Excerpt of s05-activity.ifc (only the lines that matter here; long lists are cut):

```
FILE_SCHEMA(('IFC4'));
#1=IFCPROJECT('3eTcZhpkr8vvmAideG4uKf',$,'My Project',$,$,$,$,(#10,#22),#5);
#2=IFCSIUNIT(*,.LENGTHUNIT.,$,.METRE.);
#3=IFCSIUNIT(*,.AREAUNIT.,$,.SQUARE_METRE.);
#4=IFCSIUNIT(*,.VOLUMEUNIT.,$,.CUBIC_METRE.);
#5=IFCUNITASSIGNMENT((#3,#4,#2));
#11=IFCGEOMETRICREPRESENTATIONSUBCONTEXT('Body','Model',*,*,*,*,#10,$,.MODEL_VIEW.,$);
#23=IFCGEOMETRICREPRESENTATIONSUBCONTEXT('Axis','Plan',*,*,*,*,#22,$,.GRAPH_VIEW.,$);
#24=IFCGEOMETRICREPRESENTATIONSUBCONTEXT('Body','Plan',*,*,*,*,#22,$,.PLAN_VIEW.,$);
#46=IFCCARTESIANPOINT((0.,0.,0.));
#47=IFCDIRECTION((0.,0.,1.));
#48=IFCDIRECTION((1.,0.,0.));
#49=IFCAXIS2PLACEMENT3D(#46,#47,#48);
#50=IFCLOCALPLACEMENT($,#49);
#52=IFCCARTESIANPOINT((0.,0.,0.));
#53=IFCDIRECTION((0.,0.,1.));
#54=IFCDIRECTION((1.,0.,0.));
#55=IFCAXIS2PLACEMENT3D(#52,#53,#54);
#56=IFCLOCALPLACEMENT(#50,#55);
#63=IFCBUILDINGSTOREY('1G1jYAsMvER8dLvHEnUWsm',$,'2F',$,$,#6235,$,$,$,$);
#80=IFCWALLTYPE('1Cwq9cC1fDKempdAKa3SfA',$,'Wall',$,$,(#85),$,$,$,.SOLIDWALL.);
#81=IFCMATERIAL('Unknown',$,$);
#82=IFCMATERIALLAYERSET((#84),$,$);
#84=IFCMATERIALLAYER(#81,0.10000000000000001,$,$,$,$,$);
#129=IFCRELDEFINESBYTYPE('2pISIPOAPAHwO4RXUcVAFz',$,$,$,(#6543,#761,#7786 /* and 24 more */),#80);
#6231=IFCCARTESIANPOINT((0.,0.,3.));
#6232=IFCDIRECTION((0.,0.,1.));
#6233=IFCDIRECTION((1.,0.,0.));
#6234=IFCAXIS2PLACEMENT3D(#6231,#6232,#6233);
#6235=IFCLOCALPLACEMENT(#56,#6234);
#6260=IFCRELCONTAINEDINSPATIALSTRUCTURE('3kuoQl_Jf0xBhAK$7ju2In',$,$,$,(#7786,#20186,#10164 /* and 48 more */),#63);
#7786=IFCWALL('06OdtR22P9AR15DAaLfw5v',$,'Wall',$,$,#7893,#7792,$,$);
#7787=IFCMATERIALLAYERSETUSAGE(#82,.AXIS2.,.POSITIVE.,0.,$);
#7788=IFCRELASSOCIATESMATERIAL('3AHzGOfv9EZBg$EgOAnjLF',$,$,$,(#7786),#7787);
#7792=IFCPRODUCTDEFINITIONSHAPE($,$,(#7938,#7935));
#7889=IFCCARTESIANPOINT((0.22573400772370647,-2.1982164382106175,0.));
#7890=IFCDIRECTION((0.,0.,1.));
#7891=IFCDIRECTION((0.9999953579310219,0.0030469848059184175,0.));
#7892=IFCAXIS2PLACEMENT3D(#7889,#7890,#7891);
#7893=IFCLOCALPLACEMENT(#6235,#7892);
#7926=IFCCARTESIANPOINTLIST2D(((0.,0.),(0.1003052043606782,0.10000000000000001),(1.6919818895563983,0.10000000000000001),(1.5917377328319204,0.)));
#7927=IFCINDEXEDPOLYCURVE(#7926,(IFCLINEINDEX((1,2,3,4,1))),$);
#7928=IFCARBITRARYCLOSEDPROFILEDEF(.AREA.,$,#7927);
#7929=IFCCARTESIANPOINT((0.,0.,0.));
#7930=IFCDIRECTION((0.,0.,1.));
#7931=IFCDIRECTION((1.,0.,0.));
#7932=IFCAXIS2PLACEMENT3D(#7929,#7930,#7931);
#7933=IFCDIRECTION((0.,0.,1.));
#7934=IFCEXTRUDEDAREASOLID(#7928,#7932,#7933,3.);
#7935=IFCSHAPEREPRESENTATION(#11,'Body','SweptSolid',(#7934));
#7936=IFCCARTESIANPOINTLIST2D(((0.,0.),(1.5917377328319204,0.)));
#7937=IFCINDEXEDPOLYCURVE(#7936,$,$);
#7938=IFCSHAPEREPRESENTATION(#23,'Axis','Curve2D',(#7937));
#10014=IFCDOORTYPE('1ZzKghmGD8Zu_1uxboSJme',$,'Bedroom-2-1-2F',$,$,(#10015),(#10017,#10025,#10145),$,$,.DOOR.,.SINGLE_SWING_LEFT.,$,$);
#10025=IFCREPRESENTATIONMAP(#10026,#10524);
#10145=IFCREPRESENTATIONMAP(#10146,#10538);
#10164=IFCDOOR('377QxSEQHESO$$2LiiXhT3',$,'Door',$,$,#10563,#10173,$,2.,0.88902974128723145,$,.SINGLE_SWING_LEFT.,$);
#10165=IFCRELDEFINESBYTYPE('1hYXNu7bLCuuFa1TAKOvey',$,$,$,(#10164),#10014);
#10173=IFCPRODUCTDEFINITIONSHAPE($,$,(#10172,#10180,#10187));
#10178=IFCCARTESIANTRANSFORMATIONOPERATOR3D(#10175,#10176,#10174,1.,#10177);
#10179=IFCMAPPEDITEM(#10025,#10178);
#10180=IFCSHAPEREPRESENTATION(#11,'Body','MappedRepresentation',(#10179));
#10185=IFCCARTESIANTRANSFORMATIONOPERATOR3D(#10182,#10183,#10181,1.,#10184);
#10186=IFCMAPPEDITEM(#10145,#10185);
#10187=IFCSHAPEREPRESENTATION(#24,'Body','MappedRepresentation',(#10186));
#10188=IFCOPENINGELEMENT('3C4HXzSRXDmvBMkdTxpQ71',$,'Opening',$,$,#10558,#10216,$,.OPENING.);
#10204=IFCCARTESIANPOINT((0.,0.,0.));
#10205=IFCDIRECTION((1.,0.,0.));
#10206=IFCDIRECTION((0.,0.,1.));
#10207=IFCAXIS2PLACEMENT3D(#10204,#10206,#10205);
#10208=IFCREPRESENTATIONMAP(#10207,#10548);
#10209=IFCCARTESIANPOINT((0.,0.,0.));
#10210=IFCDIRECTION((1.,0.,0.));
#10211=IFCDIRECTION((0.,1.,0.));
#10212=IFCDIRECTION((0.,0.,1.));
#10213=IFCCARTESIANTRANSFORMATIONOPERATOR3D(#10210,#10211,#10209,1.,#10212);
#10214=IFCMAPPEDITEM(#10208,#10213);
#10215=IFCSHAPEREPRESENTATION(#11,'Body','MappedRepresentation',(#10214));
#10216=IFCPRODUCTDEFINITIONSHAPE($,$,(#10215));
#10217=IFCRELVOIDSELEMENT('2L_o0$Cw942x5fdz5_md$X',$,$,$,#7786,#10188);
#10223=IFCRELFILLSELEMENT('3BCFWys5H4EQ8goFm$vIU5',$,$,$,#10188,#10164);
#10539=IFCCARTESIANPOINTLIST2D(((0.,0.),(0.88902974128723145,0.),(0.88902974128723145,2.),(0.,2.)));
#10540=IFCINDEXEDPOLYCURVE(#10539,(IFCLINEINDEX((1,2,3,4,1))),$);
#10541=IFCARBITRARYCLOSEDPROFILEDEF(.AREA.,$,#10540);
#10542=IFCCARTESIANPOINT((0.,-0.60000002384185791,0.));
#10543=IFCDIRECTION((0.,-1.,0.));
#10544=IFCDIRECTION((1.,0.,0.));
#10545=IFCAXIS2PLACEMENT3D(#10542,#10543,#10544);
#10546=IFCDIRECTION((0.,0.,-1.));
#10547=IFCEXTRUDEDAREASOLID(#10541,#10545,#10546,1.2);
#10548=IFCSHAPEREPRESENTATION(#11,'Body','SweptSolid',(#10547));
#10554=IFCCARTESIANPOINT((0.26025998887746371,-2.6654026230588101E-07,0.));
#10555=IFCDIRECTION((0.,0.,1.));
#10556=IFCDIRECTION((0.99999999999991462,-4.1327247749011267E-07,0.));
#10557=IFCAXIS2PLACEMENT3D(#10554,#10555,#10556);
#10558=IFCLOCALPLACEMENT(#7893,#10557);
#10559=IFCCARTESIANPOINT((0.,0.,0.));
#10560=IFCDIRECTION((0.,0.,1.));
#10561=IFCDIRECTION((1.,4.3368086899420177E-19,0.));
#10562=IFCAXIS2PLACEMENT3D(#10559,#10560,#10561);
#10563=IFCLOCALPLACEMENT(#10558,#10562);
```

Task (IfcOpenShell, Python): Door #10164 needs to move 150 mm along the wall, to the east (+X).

```python
import ifcopenshell
import ifcopenshell.api.geometry
import ifcopenshell.util.placement
import ifcopenshell.util.unit

model = ifcopenshell.open("s05-activity.ifc")
unit_scale = ifcopenshell.util.unit.calculate_unit_scale(model)

door = model.by_guid("377QxSEQHESO$$2LiiXhT3")
opening = door.FillsVoids[0].RelatingOpeningElement
wall = opening.VoidsElements[0].RelatingBuildingElement

wall_matrix = ifcopenshell.util.placement.get_local_placement(wall.ObjectPlacement)
shift = wall_matrix[:3, 0] * 0.15 / unit_scale
before = ifcopenshell.util.placement.get_local_placement(door.ObjectPlacement)[:3, 3].copy()

# The door is placed relative to its opening, so it follows when the opening moves.
matrix = ifcopenshell.util.placement.get_local_placement(opening.ObjectPlacement)
matrix[:3, 3] += shift
ifcopenshell.api.geometry.edit_object_placement(
    model, product=opening, matrix=matrix, is_si=False, should_transform_children=True
)

after = ifcopenshell.util.placement.get_local_placement(door.ObjectPlacement)[:3, 3]
print("door moved by", (after - before).round(3) + 0.0)

model.write("s05-activity_rev.ifc")
```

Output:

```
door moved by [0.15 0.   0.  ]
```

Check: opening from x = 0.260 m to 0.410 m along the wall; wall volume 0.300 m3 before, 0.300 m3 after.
